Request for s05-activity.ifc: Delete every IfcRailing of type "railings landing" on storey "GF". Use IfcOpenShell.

First a look at what the model holds.

```python
import ifcopenshell
import ifcopenshell.util.element

model = ifcopenshell.open("s05-activity.ifc")
print(model.schema)
storey = next(s for s in model.by_type("IfcBuildingStorey") if s.Name == "GF")
railings = [e for e in ifcopenshell.util.element.get_decomposition(storey) if e.is_a("IfcRailing")]
seen = {}
for e in railings:
    element_type = ifcopenshell.util.element.get_type(e)
    name = element_type.Name if element_type not in (None, e) else None
    seen[name] = seen.get(name, 0) + 1
for name, count in sorted(seen.items(), key=str):
    print(count, "x", name)
```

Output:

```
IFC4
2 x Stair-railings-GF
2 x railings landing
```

```python
import ifcopenshell
import ifcopenshell.api.root
import ifcopenshell.util.element

model = ifcopenshell.open("s05-activity.ifc")

storey = next(s for s in model.by_type("IfcBuildingStorey") if s.Name == "GF")
railings = [e for e in ifcopenshell.util.element.get_decomposition(storey) if e.is_a("IfcRailing")]
targets = [e for e in railings if (t := ifcopenshell.util.element.get_type(e)) not in (None, e) and t.Name == "railings landing"]

for e in targets:
    ifcopenshell.api.root.remove_product(model, product=e)
print(len(targets), "removed")

model.write("s05-activity_rev.ifc")
```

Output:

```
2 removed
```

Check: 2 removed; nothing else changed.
